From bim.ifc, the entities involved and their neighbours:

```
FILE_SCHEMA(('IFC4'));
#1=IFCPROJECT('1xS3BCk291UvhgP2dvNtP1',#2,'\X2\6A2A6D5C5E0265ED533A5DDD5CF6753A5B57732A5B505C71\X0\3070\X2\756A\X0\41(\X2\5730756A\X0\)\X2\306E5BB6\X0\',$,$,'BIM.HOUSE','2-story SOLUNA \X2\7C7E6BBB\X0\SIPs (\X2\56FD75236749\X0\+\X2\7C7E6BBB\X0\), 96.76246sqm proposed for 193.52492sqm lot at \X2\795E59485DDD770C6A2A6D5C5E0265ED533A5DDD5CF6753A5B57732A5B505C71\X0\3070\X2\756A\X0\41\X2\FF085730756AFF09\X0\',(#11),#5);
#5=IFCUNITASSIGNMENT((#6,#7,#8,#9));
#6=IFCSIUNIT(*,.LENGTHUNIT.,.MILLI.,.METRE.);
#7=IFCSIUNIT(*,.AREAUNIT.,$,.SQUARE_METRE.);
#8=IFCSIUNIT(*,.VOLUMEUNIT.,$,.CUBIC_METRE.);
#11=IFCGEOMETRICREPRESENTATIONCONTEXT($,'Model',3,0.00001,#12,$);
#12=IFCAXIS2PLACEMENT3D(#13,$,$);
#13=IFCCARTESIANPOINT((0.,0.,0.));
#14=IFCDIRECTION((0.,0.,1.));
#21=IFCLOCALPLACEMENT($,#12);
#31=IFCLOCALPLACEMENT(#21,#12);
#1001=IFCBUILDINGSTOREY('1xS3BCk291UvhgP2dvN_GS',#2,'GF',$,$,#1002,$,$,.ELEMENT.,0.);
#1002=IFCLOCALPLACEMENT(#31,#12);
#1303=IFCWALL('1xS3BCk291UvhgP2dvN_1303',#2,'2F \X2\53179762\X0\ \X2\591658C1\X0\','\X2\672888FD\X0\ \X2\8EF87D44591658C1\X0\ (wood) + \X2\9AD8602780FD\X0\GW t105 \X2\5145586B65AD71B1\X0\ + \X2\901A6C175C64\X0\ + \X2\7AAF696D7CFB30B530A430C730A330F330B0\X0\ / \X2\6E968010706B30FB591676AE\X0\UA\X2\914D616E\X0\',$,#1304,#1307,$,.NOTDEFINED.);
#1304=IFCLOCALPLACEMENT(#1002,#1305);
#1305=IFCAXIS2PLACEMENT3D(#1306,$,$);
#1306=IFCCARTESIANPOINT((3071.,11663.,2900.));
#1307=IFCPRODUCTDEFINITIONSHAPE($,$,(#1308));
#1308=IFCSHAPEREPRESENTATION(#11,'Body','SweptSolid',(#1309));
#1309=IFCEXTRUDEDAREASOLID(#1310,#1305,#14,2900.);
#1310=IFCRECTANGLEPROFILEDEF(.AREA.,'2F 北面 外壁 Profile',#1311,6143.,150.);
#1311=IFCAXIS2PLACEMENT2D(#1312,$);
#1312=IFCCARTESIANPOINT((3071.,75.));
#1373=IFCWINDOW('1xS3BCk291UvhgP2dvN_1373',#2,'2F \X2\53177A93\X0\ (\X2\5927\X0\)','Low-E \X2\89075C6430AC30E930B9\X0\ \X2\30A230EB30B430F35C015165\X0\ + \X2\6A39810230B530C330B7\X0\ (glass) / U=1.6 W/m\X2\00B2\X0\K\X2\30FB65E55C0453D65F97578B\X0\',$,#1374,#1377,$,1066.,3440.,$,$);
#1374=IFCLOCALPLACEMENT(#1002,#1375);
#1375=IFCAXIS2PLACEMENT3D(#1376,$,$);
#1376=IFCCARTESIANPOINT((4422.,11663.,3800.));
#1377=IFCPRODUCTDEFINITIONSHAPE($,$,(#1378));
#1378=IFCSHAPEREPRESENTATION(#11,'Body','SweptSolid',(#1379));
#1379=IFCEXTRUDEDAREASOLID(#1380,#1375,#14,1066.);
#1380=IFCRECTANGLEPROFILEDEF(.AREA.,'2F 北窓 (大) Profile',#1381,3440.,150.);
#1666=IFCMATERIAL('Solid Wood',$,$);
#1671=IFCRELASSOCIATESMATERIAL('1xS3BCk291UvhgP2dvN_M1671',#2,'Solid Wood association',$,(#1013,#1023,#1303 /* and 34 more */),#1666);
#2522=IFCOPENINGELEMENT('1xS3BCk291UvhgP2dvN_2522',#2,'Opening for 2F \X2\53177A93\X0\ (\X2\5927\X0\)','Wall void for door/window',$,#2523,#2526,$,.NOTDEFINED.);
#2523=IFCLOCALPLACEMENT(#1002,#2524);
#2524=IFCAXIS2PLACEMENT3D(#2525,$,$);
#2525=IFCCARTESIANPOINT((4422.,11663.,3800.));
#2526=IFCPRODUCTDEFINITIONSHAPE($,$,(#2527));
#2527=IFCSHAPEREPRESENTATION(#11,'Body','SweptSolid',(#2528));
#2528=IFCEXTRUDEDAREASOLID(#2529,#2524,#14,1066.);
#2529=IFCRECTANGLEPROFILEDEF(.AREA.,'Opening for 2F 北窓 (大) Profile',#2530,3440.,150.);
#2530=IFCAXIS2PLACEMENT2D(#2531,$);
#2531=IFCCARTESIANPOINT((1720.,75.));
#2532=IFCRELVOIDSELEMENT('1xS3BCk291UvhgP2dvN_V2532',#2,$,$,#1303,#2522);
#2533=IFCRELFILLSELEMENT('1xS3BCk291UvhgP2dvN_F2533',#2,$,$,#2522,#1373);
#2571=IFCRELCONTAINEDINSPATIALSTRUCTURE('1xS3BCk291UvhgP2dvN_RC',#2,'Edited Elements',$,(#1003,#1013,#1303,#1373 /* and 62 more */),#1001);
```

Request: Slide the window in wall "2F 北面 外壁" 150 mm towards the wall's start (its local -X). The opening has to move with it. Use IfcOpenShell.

```python
import ifcopenshell
import ifcopenshell.api.geometry
import ifcopenshell.util.placement

model = ifcopenshell.open("bim.ifc")

window = model.by_guid("1xS3BCk291UvhgP2dvN_1373")
opening = window.FillsVoids[0].RelatingOpeningElement
wall = opening.VoidsElements[0].RelatingBuildingElement

wall_matrix = ifcopenshell.util.placement.get_local_placement(wall.ObjectPlacement)
shift = wall_matrix[:3, 0] * -150.0
before = ifcopenshell.util.placement.get_local_placement(window.ObjectPlacement)[:3, 3].copy()

# The window is not placed relative to its opening, so move both.
for product in (opening, window):
    matrix = ifcopenshell.util.placement.get_local_placement(product.ObjectPlacement)
    matrix[:3, 3] += shift
    ifcopenshell.api.geometry.edit_object_placement(model, product=product, matrix=matrix, is_si=False)

after = ifcopenshell.util.placement.get_local_placement(window.ObjectPlacement)[:3, 3]
print("window moved by", (after - before).round(3) + 0.0)

model.write("bim_edited.ifc")
```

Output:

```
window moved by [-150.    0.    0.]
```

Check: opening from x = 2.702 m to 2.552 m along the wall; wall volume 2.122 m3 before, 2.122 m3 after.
